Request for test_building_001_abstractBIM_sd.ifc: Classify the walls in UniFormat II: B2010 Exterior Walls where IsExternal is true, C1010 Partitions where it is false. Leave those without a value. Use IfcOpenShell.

First a look at what the model holds.

```python
import ifcopenshell
import ifcopenshell.util.element

model = ifcopenshell.open("test_building_001_abstractBIM_sd.ifc")
print(model.schema)
print("classifications:", [c.Name for c in model.by_type("IfcClassification")])
values = [ifcopenshell.util.element.get_pset(e, "Pset_WallCommon", "IsExternal") for e in model.by_type("IfcWall")]
for value in (True, False, None):
    print("IsExternal", value, values.count(value))
```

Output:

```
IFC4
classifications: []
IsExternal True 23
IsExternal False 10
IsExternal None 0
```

```python
import ifcopenshell
import ifcopenshell.api.classification
import ifcopenshell.util.element

model = ifcopenshell.open("test_building_001_abstractBIM_sd.ifc")

system = ifcopenshell.api.classification.add_classification(model, classification="UniFormat II")

walls = model.by_type("IfcWall")
external = {e: ifcopenshell.util.element.get_pset(e, "Pset_WallCommon", "IsExternal") for e in walls}
for flag, code, name in ((True, "B2010", "Exterior Walls"), (False, "C1010", "Partitions")):
    products = [e for e in walls if external[e] is flag]
    ifcopenshell.api.classification.add_reference(
        model, products=products, classification=system, identification=code, name=name
    )
    print(code, len(products))

model.write("test_building_001_abstractBIM_sd_edited.ifc")
```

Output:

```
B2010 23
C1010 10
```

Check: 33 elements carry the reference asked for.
